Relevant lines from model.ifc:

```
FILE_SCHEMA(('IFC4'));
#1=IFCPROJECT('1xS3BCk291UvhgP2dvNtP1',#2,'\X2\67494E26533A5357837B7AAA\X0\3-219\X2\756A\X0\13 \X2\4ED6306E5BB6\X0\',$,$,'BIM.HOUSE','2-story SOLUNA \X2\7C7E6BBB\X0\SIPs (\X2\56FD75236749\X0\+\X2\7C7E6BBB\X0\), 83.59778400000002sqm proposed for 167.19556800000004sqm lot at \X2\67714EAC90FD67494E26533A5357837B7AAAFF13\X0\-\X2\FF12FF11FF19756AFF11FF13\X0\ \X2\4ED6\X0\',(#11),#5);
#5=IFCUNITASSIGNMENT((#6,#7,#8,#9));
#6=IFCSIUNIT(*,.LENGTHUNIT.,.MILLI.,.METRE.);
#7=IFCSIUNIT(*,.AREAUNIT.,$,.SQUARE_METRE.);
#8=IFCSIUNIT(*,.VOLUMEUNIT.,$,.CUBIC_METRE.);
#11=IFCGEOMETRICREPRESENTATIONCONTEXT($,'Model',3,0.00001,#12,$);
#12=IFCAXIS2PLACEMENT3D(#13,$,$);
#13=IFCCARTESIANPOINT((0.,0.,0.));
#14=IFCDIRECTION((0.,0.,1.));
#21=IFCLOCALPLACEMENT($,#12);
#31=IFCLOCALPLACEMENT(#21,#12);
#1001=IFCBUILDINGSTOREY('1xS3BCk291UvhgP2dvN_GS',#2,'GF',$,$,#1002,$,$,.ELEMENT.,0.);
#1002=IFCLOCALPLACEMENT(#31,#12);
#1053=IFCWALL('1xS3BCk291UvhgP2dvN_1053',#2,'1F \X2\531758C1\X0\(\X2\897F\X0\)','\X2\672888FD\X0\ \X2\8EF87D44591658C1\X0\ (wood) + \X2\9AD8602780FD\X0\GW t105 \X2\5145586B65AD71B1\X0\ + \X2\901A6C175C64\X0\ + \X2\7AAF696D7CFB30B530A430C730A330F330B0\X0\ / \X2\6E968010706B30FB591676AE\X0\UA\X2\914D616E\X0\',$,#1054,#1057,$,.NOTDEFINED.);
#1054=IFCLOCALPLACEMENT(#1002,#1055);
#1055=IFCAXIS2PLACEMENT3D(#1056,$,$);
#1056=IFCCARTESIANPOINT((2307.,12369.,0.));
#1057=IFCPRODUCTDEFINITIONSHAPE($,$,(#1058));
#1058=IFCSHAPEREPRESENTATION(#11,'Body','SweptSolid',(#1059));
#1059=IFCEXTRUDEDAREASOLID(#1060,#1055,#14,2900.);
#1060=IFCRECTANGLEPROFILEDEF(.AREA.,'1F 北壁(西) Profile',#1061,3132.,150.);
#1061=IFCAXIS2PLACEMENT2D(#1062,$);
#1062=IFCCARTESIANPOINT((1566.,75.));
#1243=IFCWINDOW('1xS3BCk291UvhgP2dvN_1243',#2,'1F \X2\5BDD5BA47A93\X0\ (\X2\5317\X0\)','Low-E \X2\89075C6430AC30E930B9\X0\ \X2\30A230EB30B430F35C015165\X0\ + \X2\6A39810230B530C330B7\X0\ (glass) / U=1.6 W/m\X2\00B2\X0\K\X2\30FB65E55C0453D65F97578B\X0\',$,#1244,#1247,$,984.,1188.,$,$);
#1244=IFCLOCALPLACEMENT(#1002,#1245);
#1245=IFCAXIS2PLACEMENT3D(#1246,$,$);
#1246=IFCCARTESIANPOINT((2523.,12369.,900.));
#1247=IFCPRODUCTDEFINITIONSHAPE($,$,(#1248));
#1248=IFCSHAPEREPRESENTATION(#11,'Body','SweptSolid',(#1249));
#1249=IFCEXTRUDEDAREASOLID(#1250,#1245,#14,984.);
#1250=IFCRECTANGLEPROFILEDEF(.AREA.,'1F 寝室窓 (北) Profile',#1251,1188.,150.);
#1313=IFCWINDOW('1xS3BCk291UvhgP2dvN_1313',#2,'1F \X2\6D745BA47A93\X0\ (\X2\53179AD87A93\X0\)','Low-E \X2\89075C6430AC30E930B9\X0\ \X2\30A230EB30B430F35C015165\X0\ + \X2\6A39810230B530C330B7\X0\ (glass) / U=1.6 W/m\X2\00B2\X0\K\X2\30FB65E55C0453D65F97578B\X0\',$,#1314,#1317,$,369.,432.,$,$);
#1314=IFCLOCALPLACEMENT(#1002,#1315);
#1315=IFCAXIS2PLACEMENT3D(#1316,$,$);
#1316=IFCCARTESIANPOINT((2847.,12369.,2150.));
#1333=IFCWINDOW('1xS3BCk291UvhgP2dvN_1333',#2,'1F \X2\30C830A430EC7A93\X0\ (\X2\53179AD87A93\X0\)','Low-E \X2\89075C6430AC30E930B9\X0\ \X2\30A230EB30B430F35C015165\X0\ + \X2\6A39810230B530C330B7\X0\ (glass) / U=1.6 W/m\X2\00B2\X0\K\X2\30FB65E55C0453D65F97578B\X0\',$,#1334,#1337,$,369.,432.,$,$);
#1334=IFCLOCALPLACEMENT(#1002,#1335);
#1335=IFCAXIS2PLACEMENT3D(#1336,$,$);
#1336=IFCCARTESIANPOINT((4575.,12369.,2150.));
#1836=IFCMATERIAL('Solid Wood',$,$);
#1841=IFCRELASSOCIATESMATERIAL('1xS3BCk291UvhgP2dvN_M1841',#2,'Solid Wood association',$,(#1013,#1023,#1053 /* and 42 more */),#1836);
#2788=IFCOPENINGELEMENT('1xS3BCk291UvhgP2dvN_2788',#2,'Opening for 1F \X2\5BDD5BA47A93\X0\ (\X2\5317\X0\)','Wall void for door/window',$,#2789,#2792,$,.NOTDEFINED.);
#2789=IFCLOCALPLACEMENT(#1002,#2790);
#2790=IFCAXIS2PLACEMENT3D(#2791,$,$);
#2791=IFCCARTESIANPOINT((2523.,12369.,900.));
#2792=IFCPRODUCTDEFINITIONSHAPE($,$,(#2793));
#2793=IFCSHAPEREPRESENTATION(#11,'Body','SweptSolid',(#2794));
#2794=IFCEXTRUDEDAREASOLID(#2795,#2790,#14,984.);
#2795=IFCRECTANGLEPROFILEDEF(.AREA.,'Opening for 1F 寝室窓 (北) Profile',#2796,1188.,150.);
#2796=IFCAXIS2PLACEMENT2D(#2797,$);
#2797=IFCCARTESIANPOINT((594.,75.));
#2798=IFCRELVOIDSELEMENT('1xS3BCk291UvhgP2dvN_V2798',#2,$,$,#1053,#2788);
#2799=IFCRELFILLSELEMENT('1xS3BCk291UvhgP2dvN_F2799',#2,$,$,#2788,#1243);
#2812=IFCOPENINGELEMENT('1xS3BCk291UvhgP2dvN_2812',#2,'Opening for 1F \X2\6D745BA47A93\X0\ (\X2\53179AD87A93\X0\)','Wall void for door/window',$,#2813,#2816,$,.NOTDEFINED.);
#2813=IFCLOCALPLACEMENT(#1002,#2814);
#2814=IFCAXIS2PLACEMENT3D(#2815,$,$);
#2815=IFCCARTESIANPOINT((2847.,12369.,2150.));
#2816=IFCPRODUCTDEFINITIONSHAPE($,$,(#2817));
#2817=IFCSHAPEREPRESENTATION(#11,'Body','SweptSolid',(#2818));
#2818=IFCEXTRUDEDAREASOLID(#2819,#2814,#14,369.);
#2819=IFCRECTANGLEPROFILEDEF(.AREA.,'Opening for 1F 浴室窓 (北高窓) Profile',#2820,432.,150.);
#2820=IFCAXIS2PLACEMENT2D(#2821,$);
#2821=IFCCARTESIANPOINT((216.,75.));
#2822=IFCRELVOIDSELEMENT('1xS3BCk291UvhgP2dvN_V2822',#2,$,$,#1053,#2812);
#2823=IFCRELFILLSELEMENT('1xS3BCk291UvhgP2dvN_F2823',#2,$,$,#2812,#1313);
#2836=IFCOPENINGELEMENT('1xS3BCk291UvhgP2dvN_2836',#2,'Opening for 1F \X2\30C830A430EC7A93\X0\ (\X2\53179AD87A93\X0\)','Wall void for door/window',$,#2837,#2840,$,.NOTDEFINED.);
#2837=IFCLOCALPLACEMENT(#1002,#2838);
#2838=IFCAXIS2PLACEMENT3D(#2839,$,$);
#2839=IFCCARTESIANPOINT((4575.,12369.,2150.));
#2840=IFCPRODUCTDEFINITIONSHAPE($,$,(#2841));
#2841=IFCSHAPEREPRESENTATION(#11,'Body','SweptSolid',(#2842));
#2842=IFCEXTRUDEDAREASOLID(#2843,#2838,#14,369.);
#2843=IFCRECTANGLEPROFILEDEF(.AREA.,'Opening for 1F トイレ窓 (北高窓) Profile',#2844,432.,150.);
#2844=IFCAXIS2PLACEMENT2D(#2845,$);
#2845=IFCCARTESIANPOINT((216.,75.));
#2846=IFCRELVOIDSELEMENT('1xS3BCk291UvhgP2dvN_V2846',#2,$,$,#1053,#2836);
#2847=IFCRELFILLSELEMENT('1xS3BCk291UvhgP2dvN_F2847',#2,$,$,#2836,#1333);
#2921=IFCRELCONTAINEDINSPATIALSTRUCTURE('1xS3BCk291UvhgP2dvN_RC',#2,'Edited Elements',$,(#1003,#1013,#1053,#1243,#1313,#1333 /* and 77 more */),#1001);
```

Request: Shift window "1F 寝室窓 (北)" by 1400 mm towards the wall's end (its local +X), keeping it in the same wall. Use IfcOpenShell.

```python
import ifcopenshell
import ifcopenshell.api.geometry
import ifcopenshell.util.placement

model = ifcopenshell.open("model.ifc")

window = model.by_guid("1xS3BCk291UvhgP2dvN_1243")
opening = window.FillsVoids[0].RelatingOpeningElement
wall = opening.VoidsElements[0].RelatingBuildingElement

wall_matrix = ifcopenshell.util.placement.get_local_placement(wall.ObjectPlacement)
shift = wall_matrix[:3, 0] * 1400.0
before = ifcopenshell.util.placement.get_local_placement(window.ObjectPlacement)[:3, 3].copy()

# The window is not placed relative to its opening, so move both.
for product in (opening, window):
    matrix = ifcopenshell.util.placement.get_local_placement(product.ObjectPlacement)
    matrix[:3, 3] += shift
    ifcopenshell.api.geometry.edit_object_placement(model, product=product, matrix=matrix, is_si=False)

after = ifcopenshell.util.placement.get_local_placement(window.ObjectPlacement)[:3, 3]
print("window moved by", (after - before).round(3) + 0.0)

model.write("model_edited.ifc")
```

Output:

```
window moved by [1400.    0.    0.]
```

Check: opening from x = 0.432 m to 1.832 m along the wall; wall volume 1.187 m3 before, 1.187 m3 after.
